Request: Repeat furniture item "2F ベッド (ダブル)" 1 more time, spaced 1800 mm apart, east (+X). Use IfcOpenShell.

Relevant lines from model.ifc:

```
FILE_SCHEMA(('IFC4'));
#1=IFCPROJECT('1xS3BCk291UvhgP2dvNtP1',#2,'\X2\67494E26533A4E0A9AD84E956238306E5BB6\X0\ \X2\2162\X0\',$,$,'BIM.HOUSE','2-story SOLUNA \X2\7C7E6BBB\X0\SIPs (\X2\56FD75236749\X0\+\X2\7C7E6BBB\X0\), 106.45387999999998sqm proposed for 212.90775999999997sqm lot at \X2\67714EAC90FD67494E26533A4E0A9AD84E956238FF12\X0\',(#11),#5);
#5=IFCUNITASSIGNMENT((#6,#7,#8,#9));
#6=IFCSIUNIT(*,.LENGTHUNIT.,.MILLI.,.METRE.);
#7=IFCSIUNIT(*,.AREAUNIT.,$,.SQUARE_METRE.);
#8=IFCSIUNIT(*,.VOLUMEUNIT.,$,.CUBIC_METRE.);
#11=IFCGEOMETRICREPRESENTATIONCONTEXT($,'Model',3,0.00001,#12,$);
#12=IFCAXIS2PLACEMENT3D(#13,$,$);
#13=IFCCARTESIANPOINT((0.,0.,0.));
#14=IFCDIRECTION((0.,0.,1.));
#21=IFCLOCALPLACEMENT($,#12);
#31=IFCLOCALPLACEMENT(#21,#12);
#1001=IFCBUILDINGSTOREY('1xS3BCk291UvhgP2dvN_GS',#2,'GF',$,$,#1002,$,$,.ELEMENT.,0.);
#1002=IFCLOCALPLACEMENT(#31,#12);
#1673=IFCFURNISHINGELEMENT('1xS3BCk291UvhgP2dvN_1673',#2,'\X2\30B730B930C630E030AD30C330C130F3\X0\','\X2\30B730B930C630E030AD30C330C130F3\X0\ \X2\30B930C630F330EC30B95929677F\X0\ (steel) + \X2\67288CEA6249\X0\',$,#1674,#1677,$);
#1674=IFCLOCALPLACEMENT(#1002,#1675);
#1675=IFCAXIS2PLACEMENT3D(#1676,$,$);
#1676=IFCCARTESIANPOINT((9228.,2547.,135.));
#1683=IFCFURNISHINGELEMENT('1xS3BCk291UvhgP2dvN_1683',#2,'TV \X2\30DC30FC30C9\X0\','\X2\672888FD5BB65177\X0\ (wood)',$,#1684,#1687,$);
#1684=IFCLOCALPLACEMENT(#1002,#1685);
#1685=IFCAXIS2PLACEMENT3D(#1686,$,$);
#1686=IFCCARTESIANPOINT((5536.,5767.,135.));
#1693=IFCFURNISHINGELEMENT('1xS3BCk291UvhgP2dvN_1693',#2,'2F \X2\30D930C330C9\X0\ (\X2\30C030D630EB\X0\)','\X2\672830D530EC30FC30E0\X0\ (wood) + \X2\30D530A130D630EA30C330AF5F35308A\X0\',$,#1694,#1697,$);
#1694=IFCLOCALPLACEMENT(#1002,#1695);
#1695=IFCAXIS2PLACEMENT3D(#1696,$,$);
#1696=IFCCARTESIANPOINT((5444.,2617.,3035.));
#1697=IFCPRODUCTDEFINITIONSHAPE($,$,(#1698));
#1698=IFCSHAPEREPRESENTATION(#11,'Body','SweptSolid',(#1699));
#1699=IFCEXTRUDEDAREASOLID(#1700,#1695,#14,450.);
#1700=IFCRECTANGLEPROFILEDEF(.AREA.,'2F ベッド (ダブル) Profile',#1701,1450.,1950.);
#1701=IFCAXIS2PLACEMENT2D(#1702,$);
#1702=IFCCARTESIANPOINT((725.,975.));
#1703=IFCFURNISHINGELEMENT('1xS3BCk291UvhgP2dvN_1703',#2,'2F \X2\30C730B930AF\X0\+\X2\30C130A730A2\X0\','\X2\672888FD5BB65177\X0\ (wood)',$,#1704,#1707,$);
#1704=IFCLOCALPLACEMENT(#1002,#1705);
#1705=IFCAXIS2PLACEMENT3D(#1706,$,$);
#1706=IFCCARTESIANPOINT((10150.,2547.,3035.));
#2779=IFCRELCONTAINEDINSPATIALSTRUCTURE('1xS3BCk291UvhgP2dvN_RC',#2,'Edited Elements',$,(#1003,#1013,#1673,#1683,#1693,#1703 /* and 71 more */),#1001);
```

```python
import numpy as np
import ifcopenshell
import ifcopenshell.api.geometry
import ifcopenshell.api.root
import ifcopenshell.util.element
import ifcopenshell.util.placement

model = ifcopenshell.open("model.ifc")


def reuse_history(source, copy):
    """copy_class also copies each property set's owner history, people and application; keep the originals."""
    for rel in copy.IsDefinedBy:
        if rel.is_a("IfcRelDefinesByProperties") and (history := rel.RelatingPropertyDefinition.OwnerHistory):
            rel.RelatingPropertyDefinition.OwnerHistory = source.OwnerHistory
            ifcopenshell.util.element.remove_deep2(model, history)


source = model.by_id(1693)
base = ifcopenshell.util.placement.get_local_placement(source.ObjectPlacement)
step = np.array([1.0, 0.0, 0.0]) * 1800.0

for i in range(1, 2):
    copy = ifcopenshell.api.root.copy_class(model, product=source)
    copy.Representation = ifcopenshell.util.element.copy_deep(
        model, source.Representation, exclude=["IfcGeometricRepresentationContext", "IfcRepresentationMap"]
    )
    reuse_history(source, copy)
    matrix = base.copy()
    matrix[:3, 3] += i * step
    print("added at", matrix[:3, 3].round(3) + 0.0)
    ifcopenshell.api.geometry.edit_object_placement(model, product=copy, matrix=matrix, is_si=False)

model.write("model_edited.ifc")
```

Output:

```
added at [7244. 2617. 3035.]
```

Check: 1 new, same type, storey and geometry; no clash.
